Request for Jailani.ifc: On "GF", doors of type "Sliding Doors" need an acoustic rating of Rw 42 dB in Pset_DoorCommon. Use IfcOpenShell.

First a look at what the model holds.

```python
import ifcopenshell
import ifcopenshell.util.element

model = ifcopenshell.open("Jailani.ifc")
print(model.schema)
storey = next(s for s in model.by_type("IfcBuildingStorey") if s.Name == "GF")
doors = [e for e in ifcopenshell.util.element.get_decomposition(storey) if e.is_a("IfcDoor")]
seen = {}
for e in doors:
    element_type = ifcopenshell.util.element.get_type(e)
    key = (element_type.Name if element_type != e and element_type else None, ifcopenshell.util.element.get_pset(e, "Pset_DoorCommon", "AcousticRating"))
    seen[key] = seen.get(key, 0) + 1
for (name, value), count in sorted(seen.items(), key=str):
    print(count, "x", name, "|", value)
```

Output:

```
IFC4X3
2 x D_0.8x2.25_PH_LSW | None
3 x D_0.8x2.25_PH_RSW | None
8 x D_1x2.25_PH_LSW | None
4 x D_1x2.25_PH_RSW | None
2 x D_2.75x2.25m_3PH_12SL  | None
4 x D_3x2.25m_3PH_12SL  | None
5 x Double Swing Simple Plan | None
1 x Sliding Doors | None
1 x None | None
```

```python
import ifcopenshell
import ifcopenshell.api.pset
import ifcopenshell.util.element

model = ifcopenshell.open("Jailani.ifc")

storey = next(s for s in model.by_type("IfcBuildingStorey") if s.Name == "GF")
doors = [e for e in ifcopenshell.util.element.get_decomposition(storey) if e.is_a("IfcDoor")]

count = 0
for e in doors:
    element_type = ifcopenshell.util.element.get_type(e)
    if element_type in (None, e) or element_type.Name != "Sliding Doors":
        continue
    # add_pset returns the element's existing set when there is one.
    pset = ifcopenshell.api.pset.add_pset(model, product=e, name="Pset_DoorCommon")
    ifcopenshell.api.pset.edit_pset(model, pset=pset, properties={"AcousticRating": "Rw 42 dB"})
    count += 1

print(count, "doors updated")

model.write("Jailani_rev.ifc")
```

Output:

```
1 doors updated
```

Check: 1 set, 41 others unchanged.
